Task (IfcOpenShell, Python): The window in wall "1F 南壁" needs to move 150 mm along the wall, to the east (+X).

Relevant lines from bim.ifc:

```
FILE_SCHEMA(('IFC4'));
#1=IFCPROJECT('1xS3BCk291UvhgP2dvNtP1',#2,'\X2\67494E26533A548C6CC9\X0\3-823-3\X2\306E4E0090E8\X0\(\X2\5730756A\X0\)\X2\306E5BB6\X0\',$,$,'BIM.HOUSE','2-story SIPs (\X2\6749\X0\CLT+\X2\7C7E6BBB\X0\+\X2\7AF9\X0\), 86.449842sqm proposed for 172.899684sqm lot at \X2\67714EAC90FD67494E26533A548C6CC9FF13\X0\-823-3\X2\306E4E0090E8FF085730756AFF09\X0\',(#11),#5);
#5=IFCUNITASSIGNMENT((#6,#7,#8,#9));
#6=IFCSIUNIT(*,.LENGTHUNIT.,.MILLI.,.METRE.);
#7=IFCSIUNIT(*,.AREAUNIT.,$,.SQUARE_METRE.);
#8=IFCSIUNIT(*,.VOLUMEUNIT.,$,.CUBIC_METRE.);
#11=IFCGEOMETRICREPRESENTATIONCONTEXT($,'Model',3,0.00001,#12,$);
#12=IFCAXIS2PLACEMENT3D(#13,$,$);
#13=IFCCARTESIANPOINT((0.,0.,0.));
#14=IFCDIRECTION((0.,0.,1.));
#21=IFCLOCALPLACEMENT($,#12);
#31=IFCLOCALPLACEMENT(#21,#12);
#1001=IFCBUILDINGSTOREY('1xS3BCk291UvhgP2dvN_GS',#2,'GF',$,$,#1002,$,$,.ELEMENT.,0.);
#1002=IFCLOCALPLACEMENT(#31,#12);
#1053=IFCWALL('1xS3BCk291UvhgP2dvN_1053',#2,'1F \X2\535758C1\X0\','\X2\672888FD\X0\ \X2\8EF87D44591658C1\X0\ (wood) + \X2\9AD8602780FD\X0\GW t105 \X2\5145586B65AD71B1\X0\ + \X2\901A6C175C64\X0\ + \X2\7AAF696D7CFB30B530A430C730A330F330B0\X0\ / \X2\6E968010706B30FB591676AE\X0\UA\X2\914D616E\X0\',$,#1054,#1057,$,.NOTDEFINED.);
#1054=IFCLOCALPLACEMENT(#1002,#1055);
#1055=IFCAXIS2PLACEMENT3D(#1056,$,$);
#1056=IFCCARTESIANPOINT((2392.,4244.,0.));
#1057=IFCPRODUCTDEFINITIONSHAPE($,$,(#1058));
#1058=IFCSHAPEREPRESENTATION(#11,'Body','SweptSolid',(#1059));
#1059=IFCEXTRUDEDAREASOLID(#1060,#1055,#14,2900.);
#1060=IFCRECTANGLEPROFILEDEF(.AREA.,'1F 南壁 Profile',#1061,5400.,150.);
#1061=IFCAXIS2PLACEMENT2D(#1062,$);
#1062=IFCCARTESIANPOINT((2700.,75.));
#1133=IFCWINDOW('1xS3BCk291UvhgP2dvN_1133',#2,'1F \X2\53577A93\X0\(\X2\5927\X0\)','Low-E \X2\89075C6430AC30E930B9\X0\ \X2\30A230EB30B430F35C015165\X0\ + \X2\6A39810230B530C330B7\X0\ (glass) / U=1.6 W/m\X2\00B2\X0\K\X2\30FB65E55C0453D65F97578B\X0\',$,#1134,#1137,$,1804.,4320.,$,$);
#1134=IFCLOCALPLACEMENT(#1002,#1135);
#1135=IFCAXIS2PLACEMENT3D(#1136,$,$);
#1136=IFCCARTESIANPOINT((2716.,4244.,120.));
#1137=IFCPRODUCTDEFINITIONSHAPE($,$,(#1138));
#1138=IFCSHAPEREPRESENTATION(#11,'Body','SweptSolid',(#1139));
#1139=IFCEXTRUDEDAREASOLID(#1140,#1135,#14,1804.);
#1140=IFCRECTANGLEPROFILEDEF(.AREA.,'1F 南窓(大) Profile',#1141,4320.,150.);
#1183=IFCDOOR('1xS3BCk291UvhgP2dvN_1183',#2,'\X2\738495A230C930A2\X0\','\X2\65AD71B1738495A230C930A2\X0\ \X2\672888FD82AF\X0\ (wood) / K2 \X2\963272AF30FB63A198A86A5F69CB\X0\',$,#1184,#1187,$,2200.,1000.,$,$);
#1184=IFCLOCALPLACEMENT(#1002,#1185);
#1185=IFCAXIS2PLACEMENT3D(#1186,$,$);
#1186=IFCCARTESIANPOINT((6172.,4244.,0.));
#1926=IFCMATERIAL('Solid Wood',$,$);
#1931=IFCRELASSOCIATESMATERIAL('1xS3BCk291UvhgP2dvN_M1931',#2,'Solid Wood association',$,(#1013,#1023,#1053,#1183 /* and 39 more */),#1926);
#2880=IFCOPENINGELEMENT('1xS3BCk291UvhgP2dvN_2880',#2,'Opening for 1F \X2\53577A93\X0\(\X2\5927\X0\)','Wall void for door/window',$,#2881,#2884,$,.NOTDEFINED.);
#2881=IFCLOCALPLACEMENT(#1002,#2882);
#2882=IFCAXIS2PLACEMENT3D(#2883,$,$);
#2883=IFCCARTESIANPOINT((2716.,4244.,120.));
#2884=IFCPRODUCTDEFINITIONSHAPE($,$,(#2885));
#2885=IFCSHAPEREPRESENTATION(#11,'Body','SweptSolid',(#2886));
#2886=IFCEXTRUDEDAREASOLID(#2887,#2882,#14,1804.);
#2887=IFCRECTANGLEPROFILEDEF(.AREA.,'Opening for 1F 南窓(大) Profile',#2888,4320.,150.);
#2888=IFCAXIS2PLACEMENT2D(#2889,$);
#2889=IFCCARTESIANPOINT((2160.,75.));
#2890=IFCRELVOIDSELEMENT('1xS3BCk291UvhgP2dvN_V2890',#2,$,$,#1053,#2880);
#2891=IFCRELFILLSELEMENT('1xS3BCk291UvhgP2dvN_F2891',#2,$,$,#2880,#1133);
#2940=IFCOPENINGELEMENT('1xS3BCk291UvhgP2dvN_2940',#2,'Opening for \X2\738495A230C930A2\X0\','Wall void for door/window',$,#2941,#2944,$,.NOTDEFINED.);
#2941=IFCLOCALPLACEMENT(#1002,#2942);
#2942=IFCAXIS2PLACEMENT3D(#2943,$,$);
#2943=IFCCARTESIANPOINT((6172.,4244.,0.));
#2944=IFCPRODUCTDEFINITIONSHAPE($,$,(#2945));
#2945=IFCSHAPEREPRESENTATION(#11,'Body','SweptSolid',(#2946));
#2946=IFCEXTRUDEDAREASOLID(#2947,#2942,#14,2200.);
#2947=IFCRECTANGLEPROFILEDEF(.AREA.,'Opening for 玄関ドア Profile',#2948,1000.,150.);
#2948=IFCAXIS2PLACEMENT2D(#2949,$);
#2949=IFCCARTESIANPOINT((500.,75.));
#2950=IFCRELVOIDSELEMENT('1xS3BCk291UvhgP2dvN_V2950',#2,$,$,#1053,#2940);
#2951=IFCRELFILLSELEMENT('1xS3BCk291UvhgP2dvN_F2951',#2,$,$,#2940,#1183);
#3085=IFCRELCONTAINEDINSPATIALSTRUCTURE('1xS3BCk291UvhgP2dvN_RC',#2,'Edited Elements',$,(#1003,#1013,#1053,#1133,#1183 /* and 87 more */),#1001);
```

```python
import ifcopenshell
import ifcopenshell.api.geometry
import ifcopenshell.util.placement
import ifcopenshell.util.unit

model = ifcopenshell.open("bim.ifc")
unit_scale = ifcopenshell.util.unit.calculate_unit_scale(model)

window = model.by_guid("1xS3BCk291UvhgP2dvN_1133")
opening = window.FillsVoids[0].RelatingOpeningElement
wall = opening.VoidsElements[0].RelatingBuildingElement

wall_matrix = ifcopenshell.util.placement.get_local_placement(wall.ObjectPlacement)
shift = wall_matrix[:3, 0] * 0.15 / unit_scale
before = ifcopenshell.util.placement.get_local_placement(window.ObjectPlacement)[:3, 3].copy()

# The window is not placed relative to its opening, so move both.
for product in (opening, window):
    matrix = ifcopenshell.util.placement.get_local_placement(product.ObjectPlacement)
    matrix[:3, 3] += shift
    ifcopenshell.api.geometry.edit_object_placement(model, product=product, matrix=matrix, is_si=False)

after = ifcopenshell.util.placement.get_local_placement(window.ObjectPlacement)[:3, 3]
print("window moved by", (after - before).round(3) + 0.0)

model.write("bim_rev.ifc")
```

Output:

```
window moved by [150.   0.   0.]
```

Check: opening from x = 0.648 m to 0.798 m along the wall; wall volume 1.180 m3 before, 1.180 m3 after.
